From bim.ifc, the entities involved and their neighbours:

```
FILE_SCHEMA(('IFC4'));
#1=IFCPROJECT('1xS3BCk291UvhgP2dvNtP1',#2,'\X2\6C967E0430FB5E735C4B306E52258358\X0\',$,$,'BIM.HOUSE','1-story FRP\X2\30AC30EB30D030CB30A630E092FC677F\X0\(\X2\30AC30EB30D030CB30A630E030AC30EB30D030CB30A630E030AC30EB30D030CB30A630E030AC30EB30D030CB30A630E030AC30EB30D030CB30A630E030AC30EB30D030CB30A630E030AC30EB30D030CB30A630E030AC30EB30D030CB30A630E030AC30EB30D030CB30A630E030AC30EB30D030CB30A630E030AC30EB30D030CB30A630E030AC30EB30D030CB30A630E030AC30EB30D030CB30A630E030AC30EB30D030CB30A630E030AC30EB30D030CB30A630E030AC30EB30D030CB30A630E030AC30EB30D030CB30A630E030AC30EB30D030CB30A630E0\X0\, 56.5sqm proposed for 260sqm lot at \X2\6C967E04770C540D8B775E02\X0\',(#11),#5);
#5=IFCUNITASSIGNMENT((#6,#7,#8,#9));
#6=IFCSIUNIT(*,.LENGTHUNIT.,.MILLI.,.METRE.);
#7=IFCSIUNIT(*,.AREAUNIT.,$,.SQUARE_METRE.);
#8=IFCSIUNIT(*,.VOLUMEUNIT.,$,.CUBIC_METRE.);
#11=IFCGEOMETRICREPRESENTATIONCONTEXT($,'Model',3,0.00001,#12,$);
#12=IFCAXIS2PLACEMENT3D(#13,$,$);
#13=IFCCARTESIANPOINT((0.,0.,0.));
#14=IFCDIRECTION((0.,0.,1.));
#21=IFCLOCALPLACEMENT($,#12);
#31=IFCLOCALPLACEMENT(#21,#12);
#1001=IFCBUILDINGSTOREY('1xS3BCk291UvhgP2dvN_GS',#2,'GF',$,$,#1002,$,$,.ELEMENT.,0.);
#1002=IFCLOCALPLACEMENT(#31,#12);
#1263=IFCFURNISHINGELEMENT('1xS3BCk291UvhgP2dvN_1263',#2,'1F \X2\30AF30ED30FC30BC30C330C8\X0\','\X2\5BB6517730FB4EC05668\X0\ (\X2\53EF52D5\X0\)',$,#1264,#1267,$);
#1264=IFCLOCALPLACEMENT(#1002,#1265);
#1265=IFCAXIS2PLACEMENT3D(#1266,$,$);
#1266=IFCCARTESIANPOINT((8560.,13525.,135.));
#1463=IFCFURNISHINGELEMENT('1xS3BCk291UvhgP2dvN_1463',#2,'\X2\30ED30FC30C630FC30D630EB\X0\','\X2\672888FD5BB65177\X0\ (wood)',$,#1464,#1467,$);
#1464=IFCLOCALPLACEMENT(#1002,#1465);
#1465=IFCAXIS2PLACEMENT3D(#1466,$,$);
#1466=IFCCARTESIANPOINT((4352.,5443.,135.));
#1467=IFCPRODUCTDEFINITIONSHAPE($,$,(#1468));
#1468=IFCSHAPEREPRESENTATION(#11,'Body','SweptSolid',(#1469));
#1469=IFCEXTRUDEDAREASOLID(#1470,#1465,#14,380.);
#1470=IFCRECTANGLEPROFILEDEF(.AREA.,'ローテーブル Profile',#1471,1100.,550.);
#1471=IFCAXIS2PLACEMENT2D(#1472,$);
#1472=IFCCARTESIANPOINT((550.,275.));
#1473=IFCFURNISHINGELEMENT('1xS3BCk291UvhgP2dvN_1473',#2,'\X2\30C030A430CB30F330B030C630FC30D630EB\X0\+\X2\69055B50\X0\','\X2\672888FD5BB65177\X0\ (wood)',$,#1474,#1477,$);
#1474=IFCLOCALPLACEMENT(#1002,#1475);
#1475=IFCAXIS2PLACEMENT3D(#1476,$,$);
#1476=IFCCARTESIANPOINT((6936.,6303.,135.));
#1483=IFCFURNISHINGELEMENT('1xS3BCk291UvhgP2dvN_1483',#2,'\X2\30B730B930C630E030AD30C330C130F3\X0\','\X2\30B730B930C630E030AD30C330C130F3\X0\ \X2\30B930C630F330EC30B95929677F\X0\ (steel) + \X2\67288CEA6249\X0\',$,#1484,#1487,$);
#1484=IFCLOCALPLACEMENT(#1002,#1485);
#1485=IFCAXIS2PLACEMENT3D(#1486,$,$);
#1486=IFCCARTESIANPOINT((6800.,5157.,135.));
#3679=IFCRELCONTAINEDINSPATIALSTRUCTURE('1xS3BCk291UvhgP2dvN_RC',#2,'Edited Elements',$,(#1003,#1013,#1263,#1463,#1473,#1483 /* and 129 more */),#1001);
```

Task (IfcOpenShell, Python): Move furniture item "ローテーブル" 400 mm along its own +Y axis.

```python
import ifcopenshell
import ifcopenshell.api.geometry
import ifcopenshell.util.placement
import ifcopenshell.util.unit

model = ifcopenshell.open("bim.ifc")
unit_scale = ifcopenshell.util.unit.calculate_unit_scale(model)

item = model.by_id(1463)
matrix = ifcopenshell.util.placement.get_local_placement(item.ObjectPlacement)
matrix[:3, 3] += matrix[:3, 1] * 0.4 / unit_scale
ifcopenshell.api.geometry.edit_object_placement(model, product=item, matrix=matrix, is_si=False)

print(ifcopenshell.util.placement.get_local_placement(item.ObjectPlacement).round(3) + 0.0)

model.write("bim_v2.ifc")
```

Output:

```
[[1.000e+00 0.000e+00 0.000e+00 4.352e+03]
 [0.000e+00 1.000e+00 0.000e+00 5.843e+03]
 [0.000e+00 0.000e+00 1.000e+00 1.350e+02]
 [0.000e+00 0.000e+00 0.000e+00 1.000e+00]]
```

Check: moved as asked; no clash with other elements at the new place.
